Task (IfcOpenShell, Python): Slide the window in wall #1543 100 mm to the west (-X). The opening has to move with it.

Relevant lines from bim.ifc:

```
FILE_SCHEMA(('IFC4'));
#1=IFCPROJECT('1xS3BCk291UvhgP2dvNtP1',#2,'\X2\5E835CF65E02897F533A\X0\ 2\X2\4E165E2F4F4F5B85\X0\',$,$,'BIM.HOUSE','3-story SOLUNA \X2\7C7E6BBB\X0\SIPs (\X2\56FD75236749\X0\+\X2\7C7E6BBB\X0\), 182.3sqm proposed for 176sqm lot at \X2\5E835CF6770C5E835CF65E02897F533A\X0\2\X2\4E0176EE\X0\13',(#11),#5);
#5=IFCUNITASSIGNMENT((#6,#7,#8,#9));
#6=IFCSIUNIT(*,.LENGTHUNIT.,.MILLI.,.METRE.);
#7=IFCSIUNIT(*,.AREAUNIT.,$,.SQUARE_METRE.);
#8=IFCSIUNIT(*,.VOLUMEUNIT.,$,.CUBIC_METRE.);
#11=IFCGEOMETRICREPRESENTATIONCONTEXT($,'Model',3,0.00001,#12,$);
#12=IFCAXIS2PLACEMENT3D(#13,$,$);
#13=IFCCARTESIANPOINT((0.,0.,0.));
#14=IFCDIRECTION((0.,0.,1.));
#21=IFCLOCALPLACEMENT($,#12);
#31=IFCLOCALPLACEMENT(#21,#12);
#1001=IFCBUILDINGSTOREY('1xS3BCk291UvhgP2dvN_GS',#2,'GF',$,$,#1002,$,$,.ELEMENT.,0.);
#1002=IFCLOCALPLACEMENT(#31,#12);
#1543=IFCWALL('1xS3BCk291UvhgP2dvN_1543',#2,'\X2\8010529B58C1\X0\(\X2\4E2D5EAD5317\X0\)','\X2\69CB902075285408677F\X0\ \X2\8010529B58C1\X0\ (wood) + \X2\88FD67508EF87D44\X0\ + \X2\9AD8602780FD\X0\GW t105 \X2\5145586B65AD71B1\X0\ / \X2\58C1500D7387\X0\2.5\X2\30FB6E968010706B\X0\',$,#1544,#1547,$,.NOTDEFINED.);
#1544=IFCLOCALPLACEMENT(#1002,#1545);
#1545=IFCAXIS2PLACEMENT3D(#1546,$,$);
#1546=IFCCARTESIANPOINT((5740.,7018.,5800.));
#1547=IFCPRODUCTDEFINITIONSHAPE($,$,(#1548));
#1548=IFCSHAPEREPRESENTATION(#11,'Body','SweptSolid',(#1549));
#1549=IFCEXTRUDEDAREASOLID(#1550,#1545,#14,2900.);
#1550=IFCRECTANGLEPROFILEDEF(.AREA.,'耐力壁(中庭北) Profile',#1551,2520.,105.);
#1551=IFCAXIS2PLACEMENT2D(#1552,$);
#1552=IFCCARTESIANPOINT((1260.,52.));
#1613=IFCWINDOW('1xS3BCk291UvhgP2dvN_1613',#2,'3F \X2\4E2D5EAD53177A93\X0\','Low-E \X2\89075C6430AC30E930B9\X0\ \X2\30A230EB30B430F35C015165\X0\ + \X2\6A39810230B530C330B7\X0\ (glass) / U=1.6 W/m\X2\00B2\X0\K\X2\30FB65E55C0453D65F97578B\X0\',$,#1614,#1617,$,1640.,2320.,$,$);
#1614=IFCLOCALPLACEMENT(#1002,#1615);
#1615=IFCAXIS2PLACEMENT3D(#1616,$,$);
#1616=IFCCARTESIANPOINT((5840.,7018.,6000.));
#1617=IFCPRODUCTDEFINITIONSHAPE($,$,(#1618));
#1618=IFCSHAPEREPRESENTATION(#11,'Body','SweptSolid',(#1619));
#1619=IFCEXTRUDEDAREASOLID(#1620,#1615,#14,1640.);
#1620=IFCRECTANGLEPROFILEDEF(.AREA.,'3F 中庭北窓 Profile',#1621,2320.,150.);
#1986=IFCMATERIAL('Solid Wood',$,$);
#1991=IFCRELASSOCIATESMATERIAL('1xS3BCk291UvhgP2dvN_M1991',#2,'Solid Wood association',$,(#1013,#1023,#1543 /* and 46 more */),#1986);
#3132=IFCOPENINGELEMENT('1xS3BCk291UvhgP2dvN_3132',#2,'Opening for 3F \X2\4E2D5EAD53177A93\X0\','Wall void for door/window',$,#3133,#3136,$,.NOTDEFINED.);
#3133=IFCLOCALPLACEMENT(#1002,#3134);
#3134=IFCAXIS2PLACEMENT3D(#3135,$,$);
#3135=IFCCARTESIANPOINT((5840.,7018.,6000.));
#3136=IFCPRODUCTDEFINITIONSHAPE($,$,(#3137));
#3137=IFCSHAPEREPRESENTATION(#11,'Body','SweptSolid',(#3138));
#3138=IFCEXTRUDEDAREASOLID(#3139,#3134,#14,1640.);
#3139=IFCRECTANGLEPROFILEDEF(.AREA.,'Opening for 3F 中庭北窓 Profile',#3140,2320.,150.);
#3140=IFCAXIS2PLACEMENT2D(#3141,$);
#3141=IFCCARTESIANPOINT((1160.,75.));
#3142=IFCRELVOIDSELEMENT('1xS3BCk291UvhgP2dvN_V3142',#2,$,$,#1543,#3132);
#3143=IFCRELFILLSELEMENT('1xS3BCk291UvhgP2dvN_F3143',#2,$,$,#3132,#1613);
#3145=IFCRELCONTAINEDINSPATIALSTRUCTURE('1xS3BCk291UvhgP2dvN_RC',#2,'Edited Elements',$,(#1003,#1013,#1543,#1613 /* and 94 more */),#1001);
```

```python
import ifcopenshell
import ifcopenshell.api.geometry
import ifcopenshell.util.placement

model = ifcopenshell.open("bim.ifc")

window = model.by_guid("1xS3BCk291UvhgP2dvN_1613")
opening = window.FillsVoids[0].RelatingOpeningElement
wall = opening.VoidsElements[0].RelatingBuildingElement

wall_matrix = ifcopenshell.util.placement.get_local_placement(wall.ObjectPlacement)
shift = wall_matrix[:3, 0] * -100.0
before = ifcopenshell.util.placement.get_local_placement(window.ObjectPlacement)[:3, 3].copy()

# The window is not placed relative to its opening, so move both.
for product in (opening, window):
    matrix = ifcopenshell.util.placement.get_local_placement(product.ObjectPlacement)
    matrix[:3, 3] += shift
    ifcopenshell.api.geometry.edit_object_placement(model, product=product, matrix=matrix, is_si=False)

after = ifcopenshell.util.placement.get_local_placement(window.ObjectPlacement)[:3, 3]
print("window moved by", (after - before).round(3) + 0.0)

model.write("bim_edited.ifc")
```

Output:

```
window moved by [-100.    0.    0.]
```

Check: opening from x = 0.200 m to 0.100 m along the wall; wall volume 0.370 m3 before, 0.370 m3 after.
